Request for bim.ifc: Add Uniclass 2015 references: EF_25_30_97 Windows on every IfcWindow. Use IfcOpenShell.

First a look at what the model holds.

```python
import ifcopenshell

model = ifcopenshell.open("bim.ifc")
print(model.schema)
print("classifications:", [c.Name for c in model.by_type("IfcClassification")])
for ifc_class in ("IfcDoor", "IfcRoof", "IfcStair", "IfcWall", "IfcWindow"):
    print(ifc_class, len(model.by_type(ifc_class)))
```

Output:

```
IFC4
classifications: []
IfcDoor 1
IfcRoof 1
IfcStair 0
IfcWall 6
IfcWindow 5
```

```python
import ifcopenshell
import ifcopenshell.api.classification

model = ifcopenshell.open("bim.ifc")

system = ifcopenshell.api.classification.add_classification(model, classification="Uniclass 2015")

codes = {
    "IfcWindow": ("EF_25_30_97", "Windows"),
}
for ifc_class, (code, name) in codes.items():
    products = model.by_type(ifc_class)
    ifcopenshell.api.classification.add_reference(
        model, products=products, classification=system, identification=code, name=name
    )
    print(code, len(products))

model.write("bim_v2.ifc")
```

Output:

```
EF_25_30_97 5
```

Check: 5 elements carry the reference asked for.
